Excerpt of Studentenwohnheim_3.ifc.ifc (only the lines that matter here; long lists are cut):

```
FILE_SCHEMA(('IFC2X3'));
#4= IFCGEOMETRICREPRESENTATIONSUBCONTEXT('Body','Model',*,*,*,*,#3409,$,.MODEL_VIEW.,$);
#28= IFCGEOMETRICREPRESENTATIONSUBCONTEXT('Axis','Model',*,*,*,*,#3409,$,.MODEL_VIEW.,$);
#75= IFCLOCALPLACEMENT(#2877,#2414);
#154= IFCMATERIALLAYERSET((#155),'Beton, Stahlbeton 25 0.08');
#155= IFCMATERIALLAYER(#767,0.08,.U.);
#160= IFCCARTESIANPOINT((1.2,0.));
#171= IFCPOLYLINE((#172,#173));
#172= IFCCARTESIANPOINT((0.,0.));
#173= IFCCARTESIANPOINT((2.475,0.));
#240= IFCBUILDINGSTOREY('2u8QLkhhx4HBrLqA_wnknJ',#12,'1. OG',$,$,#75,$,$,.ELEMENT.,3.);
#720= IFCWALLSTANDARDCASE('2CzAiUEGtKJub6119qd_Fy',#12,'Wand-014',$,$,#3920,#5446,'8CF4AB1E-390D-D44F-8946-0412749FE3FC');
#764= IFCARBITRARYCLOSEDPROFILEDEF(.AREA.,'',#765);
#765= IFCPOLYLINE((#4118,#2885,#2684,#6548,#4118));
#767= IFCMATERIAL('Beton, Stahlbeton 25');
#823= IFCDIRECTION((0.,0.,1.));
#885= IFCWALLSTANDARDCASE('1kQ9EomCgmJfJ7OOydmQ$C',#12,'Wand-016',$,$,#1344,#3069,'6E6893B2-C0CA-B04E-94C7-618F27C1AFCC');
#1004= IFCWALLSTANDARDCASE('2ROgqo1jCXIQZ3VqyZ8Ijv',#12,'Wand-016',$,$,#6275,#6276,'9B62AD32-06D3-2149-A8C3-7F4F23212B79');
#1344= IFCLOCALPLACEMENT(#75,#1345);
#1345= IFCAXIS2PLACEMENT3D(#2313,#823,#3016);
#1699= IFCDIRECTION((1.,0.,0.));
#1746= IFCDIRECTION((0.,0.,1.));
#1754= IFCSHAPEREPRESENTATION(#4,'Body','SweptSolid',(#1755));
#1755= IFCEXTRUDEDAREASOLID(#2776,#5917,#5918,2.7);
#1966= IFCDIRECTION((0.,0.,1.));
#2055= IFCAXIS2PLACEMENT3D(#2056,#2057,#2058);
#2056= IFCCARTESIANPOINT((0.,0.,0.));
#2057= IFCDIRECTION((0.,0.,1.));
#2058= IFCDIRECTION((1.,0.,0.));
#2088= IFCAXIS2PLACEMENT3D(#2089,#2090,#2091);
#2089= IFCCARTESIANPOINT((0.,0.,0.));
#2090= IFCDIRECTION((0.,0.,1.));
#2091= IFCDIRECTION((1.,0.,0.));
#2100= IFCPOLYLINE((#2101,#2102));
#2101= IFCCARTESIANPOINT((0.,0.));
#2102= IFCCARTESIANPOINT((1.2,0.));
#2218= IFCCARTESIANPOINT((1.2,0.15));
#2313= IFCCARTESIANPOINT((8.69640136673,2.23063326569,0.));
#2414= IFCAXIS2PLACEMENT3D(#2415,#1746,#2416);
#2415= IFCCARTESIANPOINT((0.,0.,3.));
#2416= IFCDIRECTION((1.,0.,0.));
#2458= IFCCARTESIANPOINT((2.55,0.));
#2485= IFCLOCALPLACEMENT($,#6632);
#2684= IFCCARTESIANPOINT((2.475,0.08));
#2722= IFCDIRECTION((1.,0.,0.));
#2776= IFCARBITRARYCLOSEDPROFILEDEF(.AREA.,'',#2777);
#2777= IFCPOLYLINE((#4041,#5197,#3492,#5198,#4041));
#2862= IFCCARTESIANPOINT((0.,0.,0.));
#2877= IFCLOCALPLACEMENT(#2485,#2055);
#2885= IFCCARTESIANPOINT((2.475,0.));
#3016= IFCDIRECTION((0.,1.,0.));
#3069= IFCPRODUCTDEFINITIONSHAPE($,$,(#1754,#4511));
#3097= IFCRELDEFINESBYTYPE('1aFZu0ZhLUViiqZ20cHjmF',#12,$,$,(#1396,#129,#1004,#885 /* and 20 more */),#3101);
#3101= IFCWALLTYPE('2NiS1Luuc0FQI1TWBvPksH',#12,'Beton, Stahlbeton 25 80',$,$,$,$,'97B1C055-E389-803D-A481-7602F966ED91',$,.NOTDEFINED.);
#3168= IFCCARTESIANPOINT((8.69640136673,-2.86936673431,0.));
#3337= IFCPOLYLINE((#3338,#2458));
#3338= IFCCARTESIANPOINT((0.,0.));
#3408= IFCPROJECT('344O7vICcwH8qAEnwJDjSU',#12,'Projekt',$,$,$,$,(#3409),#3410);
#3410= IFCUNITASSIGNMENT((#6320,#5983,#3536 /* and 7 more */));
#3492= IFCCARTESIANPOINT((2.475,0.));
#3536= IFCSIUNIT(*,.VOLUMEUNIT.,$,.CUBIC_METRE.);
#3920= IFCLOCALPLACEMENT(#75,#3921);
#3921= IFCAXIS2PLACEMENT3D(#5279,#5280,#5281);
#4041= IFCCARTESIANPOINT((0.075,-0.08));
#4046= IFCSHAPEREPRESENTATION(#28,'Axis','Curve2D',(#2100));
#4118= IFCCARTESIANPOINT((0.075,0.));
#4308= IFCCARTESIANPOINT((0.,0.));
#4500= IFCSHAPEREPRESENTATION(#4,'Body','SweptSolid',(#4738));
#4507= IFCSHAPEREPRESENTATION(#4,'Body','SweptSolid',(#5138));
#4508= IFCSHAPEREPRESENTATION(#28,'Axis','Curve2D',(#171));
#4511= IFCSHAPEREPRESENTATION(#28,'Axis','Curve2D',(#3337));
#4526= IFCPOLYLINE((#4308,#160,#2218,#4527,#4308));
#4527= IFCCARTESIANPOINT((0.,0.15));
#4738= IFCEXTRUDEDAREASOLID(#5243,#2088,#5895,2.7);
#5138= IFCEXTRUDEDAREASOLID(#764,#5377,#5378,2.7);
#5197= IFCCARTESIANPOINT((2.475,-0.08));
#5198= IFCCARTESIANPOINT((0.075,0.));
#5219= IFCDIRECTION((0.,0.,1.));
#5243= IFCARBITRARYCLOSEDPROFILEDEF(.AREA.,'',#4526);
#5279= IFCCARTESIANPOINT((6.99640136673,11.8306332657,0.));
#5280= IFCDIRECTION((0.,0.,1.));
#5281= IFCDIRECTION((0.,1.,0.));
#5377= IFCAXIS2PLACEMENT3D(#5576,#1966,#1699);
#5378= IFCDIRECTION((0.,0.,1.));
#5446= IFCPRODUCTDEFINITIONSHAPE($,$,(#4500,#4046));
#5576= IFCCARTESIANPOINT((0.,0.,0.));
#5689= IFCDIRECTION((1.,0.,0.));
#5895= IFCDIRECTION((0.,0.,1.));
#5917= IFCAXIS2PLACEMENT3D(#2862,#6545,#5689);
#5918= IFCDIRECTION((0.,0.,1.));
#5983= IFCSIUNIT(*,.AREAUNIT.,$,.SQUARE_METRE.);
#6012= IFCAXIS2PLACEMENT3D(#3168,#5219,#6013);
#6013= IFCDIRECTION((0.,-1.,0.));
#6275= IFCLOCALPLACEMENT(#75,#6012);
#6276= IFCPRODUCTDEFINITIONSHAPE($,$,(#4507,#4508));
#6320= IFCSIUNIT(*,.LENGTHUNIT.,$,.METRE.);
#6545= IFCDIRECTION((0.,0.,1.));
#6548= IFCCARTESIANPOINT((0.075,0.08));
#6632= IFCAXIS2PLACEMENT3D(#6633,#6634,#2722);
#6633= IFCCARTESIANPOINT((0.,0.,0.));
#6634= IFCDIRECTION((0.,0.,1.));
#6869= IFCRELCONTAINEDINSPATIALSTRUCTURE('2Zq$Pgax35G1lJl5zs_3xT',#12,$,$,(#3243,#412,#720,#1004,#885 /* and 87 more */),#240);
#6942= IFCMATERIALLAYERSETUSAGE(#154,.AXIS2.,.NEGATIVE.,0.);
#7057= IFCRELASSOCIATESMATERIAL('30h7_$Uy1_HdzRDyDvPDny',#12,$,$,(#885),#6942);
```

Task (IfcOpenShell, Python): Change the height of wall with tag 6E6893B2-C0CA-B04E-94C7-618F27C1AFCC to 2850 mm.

```python
import ifcopenshell
import ifcopenshell.geom
import ifcopenshell.util.representation
import ifcopenshell.util.shape
import ifcopenshell.util.unit

model = ifcopenshell.open("Studentenwohnheim_3.ifc.ifc")
unit_scale = ifcopenshell.util.unit.calculate_unit_scale(model)
settings = ifcopenshell.geom.settings()


def volume(element):
    """Net volume in cubic metres, openings subtracted."""
    shape = ifcopenshell.geom.create_shape(settings, element)
    return ifcopenshell.util.shape.get_volume(shape.geometry)


wall = model.by_guid("1kQ9EomCgmJfJ7OOydmQ$C")
before = volume(wall)

body = ifcopenshell.util.representation.get_representation(wall, "Model", "Body")
solid = body.Items[0]
old_height = solid.Depth
solid.Depth = 2.85 / unit_scale
after = volume(wall)

print(f"height {old_height:g} -> {solid.Depth:g}, volume {before:.3f} -> {after:.3f} m3")

model.write("Studentenwohnheim_3.ifc_edited.ifc")
```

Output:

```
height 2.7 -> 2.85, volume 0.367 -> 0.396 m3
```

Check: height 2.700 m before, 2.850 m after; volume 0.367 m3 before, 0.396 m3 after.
